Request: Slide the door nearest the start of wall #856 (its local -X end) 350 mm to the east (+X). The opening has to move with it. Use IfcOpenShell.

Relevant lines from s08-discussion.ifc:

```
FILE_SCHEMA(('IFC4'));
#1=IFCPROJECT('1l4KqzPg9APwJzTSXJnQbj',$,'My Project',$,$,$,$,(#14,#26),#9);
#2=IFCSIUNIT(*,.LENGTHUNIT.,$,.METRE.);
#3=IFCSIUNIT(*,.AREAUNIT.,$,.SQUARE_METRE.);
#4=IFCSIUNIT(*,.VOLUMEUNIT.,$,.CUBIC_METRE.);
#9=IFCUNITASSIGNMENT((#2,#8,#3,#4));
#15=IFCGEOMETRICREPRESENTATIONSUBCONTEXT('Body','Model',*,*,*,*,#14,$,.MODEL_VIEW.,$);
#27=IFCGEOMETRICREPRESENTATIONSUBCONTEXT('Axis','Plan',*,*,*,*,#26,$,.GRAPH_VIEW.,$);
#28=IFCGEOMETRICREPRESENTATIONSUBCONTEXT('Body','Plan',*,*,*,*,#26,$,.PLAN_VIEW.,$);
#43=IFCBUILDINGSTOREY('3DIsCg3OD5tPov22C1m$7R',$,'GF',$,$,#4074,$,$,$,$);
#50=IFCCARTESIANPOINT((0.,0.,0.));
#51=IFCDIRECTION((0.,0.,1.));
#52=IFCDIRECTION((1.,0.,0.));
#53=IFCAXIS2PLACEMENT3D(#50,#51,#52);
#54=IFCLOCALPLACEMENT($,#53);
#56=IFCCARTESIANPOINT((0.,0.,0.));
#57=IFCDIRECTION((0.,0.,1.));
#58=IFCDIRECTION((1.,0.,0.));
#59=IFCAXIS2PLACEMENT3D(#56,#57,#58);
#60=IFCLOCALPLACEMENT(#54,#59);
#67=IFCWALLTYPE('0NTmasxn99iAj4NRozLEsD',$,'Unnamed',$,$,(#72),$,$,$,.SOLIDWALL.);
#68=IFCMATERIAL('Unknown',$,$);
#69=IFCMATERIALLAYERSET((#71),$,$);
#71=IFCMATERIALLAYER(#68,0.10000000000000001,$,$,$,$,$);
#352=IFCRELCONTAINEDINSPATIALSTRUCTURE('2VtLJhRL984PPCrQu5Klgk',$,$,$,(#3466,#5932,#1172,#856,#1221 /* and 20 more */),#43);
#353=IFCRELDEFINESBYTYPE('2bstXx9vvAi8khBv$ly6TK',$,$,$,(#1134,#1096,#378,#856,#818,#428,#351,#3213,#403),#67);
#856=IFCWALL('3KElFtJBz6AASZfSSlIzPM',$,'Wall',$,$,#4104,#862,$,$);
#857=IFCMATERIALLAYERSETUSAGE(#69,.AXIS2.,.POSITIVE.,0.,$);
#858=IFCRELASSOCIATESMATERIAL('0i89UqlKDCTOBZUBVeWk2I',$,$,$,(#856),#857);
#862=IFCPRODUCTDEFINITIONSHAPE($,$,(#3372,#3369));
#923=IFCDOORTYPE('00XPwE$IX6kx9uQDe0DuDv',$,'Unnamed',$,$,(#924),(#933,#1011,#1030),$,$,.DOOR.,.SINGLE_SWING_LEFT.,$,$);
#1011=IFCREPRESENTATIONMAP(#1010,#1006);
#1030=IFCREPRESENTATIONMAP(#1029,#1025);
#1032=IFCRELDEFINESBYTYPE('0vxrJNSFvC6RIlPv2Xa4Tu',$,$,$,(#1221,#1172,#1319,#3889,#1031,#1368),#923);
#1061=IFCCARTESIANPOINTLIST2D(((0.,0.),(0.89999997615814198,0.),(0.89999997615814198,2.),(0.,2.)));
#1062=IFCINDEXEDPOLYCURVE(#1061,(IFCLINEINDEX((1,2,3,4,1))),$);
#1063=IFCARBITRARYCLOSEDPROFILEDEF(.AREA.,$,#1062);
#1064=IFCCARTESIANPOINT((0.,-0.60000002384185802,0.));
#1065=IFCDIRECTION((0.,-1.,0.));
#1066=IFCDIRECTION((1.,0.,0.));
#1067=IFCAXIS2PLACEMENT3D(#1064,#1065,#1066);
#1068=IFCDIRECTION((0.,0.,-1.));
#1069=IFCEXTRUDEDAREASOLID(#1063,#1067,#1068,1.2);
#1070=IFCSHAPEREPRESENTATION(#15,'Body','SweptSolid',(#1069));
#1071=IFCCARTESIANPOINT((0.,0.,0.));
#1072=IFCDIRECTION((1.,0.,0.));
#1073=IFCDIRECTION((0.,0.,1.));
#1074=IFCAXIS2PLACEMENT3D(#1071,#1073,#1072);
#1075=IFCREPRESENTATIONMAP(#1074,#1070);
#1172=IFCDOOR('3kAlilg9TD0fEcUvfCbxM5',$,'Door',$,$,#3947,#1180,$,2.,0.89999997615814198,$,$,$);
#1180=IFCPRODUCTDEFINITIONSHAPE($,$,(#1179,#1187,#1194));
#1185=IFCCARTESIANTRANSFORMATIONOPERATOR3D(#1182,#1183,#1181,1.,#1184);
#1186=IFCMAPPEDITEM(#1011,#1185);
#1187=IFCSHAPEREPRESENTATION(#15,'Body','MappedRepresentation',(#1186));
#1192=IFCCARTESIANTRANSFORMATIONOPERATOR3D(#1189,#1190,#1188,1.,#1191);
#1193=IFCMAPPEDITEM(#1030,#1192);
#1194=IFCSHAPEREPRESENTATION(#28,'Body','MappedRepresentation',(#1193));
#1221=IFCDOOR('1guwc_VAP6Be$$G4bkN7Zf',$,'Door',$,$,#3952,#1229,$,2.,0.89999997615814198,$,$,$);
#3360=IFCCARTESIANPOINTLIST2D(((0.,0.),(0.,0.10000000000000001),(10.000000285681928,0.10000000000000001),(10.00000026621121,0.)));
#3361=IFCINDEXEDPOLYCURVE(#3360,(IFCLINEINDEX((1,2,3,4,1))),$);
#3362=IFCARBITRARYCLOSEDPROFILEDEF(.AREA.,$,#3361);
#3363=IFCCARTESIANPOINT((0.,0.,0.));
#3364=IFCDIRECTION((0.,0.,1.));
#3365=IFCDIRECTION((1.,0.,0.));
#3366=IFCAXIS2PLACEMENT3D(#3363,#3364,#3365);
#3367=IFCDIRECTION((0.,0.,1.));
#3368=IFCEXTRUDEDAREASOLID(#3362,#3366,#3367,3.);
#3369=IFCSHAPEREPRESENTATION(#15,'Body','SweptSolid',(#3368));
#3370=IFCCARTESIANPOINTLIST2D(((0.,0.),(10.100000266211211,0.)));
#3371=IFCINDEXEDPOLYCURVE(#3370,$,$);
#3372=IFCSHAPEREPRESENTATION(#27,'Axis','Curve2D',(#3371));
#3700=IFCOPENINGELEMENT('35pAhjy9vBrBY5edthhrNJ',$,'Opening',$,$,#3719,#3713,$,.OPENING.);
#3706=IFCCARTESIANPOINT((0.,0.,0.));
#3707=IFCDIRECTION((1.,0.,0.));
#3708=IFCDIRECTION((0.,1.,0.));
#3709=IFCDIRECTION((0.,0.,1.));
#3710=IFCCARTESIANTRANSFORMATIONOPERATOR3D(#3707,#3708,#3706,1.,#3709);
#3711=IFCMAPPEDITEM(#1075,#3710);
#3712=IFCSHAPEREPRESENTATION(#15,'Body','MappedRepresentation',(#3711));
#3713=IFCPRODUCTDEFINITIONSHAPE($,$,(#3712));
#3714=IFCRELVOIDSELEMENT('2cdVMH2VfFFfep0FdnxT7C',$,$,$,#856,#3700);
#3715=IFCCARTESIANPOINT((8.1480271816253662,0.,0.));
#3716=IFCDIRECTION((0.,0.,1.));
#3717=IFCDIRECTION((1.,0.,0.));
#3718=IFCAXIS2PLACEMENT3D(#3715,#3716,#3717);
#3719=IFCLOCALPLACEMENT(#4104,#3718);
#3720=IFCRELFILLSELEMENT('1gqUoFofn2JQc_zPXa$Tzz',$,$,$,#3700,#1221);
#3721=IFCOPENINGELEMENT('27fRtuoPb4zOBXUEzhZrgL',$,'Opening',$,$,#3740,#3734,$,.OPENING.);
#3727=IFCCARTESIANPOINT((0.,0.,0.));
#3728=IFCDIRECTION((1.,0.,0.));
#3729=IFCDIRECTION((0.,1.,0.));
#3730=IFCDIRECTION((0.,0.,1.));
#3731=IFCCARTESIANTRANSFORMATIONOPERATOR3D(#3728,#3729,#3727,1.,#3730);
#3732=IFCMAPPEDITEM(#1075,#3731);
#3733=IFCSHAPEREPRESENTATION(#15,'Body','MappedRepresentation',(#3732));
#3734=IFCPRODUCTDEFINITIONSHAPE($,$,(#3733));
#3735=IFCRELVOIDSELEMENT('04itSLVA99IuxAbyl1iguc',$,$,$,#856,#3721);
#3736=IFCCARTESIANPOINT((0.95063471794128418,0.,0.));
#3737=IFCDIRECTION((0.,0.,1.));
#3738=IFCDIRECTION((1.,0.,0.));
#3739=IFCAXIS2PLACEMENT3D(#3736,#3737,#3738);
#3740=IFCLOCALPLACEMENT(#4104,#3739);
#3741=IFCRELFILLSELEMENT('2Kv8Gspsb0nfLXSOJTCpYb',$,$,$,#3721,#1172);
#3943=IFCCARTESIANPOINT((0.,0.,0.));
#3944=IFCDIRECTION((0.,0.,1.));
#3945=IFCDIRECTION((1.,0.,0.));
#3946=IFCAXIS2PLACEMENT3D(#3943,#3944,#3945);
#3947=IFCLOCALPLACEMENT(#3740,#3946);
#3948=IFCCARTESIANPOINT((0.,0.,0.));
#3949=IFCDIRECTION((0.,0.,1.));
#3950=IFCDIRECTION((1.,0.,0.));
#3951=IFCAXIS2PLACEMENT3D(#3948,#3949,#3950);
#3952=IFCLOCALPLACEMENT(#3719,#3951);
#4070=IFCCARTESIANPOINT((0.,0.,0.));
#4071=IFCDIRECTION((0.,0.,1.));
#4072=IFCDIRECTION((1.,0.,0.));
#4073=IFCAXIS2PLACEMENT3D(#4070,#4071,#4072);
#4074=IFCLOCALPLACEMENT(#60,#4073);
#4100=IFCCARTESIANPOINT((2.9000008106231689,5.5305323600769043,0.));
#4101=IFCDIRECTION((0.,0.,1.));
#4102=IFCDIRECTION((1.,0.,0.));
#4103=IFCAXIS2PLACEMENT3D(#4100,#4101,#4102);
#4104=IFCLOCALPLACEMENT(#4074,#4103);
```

```python
import ifcopenshell
import ifcopenshell.api.geometry
import ifcopenshell.util.placement

model = ifcopenshell.open("s08-discussion.ifc")

door = model.by_guid("3kAlilg9TD0fEcUvfCbxM5")
opening = door.FillsVoids[0].RelatingOpeningElement
wall = opening.VoidsElements[0].RelatingBuildingElement

wall_matrix = ifcopenshell.util.placement.get_local_placement(wall.ObjectPlacement)
shift = wall_matrix[:3, 0] * 0.35
before = ifcopenshell.util.placement.get_local_placement(door.ObjectPlacement)[:3, 3].copy()

# The door is placed relative to its opening, so it follows when the opening moves.
matrix = ifcopenshell.util.placement.get_local_placement(opening.ObjectPlacement)
matrix[:3, 3] += shift
ifcopenshell.api.geometry.edit_object_placement(
    model, product=opening, matrix=matrix, is_si=False, should_transform_children=True
)

after = ifcopenshell.util.placement.get_local_placement(door.ObjectPlacement)[:3, 3]
print("door moved by", (after - before).round(3) + 0.0)

model.write("s08-discussion_edited.ifc")
```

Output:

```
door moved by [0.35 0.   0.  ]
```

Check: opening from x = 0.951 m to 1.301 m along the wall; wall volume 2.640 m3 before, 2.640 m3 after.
